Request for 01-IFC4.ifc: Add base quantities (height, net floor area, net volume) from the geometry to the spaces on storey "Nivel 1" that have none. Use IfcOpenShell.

First a look at what the model holds.

```python
import ifcopenshell
import ifcopenshell.util.element
import ifcopenshell.util.unit

model = ifcopenshell.open("01-IFC4.ifc")
print(model.schema)
for unit_type in ("LENGTHUNIT", "AREAUNIT", "VOLUMEUNIT"):
    print(unit_type, ifcopenshell.util.unit.calculate_unit_scale(model, unit_type))
storey = next(s for s in model.by_type("IfcBuildingStorey") if s.Name == "Nivel 1")
spaces = [e for e in ifcopenshell.util.element.get_decomposition(storey) if e.is_a("IfcSpace")]
for e in sorted(spaces, key=lambda e: e.id()):
    print(e.id(), e.is_a(), e.Name, list(ifcopenshell.util.element.get_psets(e, qtos_only=True)), sep=" | ")
```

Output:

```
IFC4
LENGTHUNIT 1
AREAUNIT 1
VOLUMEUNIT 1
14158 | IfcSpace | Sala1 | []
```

```python
import ifcopenshell
import ifcopenshell.api.pset
import ifcopenshell.geom
import ifcopenshell.util.element
import ifcopenshell.util.shape
import ifcopenshell.util.unit

model = ifcopenshell.open("01-IFC4.ifc")
unit_scale = ifcopenshell.util.unit.calculate_unit_scale(model)
area_scale = ifcopenshell.util.unit.calculate_unit_scale(model, "AREAUNIT")
volume_scale = ifcopenshell.util.unit.calculate_unit_scale(model, "VOLUMEUNIT")
settings = ifcopenshell.geom.settings()

storey = next(s for s in model.by_type("IfcBuildingStorey") if s.Name == "Nivel 1")
spaces = [e for e in ifcopenshell.util.element.get_decomposition(storey) if e.is_a("IfcSpace")]

for e in sorted(spaces, key=lambda e: e.id()):
    if ifcopenshell.util.element.get_psets(e, qtos_only=True, should_inherit=False):
        continue
    # Geometry comes back in metres, in the element's own axes.
    shape = ifcopenshell.geom.create_shape(settings, e)
    values = {
        "Height": ifcopenshell.util.shape.get_z(shape.geometry) / unit_scale,
        "NetFloorArea": ifcopenshell.util.shape.get_footprint_area(shape.geometry) / area_scale,
        "NetVolume": ifcopenshell.util.shape.get_volume(shape.geometry) / volume_scale,
    }
    qto = ifcopenshell.api.pset.add_qto(model, product=e, name="Qto_SpaceBaseQuantities")
    ifcopenshell.api.pset.edit_qto(model, qto=qto, properties=values)
    print(e.id(), {k: round(v, 3) for k, v in values.items()})

model.write("01-IFC4_rev.ifc")
```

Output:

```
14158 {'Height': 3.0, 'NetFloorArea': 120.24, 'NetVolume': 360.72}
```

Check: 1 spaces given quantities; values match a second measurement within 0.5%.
